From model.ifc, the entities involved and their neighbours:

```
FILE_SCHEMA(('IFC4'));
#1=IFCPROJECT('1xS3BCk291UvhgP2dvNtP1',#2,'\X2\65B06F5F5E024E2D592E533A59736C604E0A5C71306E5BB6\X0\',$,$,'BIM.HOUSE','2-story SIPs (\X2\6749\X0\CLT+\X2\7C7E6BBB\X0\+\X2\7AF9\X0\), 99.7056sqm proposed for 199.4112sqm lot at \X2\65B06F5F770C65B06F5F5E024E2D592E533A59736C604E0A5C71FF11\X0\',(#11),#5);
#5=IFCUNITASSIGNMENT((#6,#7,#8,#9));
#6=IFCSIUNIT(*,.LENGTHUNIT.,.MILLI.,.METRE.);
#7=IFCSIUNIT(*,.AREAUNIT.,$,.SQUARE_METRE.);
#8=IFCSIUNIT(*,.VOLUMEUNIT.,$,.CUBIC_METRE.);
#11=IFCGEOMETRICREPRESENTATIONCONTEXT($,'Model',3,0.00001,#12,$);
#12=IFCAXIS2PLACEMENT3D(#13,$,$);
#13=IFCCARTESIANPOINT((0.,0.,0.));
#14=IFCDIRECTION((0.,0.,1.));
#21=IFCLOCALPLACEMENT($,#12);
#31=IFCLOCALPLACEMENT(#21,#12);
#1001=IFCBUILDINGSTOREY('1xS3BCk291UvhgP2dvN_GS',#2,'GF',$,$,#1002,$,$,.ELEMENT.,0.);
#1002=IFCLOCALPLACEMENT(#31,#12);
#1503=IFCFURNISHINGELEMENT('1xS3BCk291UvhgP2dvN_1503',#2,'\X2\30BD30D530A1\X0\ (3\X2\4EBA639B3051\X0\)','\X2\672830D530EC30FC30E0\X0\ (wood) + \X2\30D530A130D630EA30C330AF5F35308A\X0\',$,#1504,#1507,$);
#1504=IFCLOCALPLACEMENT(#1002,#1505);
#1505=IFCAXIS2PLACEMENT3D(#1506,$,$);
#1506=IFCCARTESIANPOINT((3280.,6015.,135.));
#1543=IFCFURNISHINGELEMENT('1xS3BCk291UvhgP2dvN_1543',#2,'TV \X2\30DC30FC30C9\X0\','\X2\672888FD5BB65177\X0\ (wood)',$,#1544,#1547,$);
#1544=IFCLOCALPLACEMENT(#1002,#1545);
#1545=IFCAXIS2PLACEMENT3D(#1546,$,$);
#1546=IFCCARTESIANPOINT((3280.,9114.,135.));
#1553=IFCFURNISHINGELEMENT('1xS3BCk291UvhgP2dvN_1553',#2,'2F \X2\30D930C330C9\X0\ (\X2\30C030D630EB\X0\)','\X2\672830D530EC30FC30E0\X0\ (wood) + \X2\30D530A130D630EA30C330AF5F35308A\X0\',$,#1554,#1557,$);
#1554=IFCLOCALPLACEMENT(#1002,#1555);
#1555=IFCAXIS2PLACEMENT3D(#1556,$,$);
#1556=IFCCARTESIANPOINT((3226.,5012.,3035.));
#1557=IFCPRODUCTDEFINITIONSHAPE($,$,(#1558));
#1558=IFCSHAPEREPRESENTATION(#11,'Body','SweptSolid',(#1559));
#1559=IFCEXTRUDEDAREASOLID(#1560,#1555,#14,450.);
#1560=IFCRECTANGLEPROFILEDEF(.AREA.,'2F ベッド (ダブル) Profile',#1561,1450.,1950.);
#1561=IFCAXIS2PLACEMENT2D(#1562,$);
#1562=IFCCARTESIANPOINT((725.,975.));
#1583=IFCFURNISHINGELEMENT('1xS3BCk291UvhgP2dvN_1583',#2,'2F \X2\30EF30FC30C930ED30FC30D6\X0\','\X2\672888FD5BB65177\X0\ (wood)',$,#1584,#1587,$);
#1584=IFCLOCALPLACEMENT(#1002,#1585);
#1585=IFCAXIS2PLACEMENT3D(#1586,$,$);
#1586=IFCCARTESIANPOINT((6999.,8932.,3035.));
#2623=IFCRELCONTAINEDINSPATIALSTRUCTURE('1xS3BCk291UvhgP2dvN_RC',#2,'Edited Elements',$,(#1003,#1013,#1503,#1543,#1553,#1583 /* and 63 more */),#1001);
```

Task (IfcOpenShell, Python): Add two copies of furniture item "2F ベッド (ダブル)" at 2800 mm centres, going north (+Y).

```python
import numpy as np
import ifcopenshell
import ifcopenshell.api.geometry
import ifcopenshell.api.root
import ifcopenshell.util.element
import ifcopenshell.util.placement

model = ifcopenshell.open("model.ifc")


def reuse_history(source, copy):
    """copy_class also copies each property set's owner history, people and application; keep the originals."""
    for rel in copy.IsDefinedBy:
        if rel.is_a("IfcRelDefinesByProperties") and (history := rel.RelatingPropertyDefinition.OwnerHistory):
            rel.RelatingPropertyDefinition.OwnerHistory = source.OwnerHistory
            ifcopenshell.util.element.remove_deep2(model, history)


source = model.by_guid("1xS3BCk291UvhgP2dvN_1553")
base = ifcopenshell.util.placement.get_local_placement(source.ObjectPlacement)
step = np.array([0.0, 1.0, 0.0]) * 2800.0

for i in range(1, 3):
    copy = ifcopenshell.api.root.copy_class(model, product=source)
    copy.Representation = ifcopenshell.util.element.copy_deep(
        model, source.Representation, exclude=["IfcGeometricRepresentationContext", "IfcRepresentationMap"]
    )
    reuse_history(source, copy)
    matrix = base.copy()
    matrix[:3, 3] += i * step
    print("added at", matrix[:3, 3].round(3) + 0.0)
    ifcopenshell.api.geometry.edit_object_placement(model, product=copy, matrix=matrix, is_si=False)

model.write("model_rev.ifc")
```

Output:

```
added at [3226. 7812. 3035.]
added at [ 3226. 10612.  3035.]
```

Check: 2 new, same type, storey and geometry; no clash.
